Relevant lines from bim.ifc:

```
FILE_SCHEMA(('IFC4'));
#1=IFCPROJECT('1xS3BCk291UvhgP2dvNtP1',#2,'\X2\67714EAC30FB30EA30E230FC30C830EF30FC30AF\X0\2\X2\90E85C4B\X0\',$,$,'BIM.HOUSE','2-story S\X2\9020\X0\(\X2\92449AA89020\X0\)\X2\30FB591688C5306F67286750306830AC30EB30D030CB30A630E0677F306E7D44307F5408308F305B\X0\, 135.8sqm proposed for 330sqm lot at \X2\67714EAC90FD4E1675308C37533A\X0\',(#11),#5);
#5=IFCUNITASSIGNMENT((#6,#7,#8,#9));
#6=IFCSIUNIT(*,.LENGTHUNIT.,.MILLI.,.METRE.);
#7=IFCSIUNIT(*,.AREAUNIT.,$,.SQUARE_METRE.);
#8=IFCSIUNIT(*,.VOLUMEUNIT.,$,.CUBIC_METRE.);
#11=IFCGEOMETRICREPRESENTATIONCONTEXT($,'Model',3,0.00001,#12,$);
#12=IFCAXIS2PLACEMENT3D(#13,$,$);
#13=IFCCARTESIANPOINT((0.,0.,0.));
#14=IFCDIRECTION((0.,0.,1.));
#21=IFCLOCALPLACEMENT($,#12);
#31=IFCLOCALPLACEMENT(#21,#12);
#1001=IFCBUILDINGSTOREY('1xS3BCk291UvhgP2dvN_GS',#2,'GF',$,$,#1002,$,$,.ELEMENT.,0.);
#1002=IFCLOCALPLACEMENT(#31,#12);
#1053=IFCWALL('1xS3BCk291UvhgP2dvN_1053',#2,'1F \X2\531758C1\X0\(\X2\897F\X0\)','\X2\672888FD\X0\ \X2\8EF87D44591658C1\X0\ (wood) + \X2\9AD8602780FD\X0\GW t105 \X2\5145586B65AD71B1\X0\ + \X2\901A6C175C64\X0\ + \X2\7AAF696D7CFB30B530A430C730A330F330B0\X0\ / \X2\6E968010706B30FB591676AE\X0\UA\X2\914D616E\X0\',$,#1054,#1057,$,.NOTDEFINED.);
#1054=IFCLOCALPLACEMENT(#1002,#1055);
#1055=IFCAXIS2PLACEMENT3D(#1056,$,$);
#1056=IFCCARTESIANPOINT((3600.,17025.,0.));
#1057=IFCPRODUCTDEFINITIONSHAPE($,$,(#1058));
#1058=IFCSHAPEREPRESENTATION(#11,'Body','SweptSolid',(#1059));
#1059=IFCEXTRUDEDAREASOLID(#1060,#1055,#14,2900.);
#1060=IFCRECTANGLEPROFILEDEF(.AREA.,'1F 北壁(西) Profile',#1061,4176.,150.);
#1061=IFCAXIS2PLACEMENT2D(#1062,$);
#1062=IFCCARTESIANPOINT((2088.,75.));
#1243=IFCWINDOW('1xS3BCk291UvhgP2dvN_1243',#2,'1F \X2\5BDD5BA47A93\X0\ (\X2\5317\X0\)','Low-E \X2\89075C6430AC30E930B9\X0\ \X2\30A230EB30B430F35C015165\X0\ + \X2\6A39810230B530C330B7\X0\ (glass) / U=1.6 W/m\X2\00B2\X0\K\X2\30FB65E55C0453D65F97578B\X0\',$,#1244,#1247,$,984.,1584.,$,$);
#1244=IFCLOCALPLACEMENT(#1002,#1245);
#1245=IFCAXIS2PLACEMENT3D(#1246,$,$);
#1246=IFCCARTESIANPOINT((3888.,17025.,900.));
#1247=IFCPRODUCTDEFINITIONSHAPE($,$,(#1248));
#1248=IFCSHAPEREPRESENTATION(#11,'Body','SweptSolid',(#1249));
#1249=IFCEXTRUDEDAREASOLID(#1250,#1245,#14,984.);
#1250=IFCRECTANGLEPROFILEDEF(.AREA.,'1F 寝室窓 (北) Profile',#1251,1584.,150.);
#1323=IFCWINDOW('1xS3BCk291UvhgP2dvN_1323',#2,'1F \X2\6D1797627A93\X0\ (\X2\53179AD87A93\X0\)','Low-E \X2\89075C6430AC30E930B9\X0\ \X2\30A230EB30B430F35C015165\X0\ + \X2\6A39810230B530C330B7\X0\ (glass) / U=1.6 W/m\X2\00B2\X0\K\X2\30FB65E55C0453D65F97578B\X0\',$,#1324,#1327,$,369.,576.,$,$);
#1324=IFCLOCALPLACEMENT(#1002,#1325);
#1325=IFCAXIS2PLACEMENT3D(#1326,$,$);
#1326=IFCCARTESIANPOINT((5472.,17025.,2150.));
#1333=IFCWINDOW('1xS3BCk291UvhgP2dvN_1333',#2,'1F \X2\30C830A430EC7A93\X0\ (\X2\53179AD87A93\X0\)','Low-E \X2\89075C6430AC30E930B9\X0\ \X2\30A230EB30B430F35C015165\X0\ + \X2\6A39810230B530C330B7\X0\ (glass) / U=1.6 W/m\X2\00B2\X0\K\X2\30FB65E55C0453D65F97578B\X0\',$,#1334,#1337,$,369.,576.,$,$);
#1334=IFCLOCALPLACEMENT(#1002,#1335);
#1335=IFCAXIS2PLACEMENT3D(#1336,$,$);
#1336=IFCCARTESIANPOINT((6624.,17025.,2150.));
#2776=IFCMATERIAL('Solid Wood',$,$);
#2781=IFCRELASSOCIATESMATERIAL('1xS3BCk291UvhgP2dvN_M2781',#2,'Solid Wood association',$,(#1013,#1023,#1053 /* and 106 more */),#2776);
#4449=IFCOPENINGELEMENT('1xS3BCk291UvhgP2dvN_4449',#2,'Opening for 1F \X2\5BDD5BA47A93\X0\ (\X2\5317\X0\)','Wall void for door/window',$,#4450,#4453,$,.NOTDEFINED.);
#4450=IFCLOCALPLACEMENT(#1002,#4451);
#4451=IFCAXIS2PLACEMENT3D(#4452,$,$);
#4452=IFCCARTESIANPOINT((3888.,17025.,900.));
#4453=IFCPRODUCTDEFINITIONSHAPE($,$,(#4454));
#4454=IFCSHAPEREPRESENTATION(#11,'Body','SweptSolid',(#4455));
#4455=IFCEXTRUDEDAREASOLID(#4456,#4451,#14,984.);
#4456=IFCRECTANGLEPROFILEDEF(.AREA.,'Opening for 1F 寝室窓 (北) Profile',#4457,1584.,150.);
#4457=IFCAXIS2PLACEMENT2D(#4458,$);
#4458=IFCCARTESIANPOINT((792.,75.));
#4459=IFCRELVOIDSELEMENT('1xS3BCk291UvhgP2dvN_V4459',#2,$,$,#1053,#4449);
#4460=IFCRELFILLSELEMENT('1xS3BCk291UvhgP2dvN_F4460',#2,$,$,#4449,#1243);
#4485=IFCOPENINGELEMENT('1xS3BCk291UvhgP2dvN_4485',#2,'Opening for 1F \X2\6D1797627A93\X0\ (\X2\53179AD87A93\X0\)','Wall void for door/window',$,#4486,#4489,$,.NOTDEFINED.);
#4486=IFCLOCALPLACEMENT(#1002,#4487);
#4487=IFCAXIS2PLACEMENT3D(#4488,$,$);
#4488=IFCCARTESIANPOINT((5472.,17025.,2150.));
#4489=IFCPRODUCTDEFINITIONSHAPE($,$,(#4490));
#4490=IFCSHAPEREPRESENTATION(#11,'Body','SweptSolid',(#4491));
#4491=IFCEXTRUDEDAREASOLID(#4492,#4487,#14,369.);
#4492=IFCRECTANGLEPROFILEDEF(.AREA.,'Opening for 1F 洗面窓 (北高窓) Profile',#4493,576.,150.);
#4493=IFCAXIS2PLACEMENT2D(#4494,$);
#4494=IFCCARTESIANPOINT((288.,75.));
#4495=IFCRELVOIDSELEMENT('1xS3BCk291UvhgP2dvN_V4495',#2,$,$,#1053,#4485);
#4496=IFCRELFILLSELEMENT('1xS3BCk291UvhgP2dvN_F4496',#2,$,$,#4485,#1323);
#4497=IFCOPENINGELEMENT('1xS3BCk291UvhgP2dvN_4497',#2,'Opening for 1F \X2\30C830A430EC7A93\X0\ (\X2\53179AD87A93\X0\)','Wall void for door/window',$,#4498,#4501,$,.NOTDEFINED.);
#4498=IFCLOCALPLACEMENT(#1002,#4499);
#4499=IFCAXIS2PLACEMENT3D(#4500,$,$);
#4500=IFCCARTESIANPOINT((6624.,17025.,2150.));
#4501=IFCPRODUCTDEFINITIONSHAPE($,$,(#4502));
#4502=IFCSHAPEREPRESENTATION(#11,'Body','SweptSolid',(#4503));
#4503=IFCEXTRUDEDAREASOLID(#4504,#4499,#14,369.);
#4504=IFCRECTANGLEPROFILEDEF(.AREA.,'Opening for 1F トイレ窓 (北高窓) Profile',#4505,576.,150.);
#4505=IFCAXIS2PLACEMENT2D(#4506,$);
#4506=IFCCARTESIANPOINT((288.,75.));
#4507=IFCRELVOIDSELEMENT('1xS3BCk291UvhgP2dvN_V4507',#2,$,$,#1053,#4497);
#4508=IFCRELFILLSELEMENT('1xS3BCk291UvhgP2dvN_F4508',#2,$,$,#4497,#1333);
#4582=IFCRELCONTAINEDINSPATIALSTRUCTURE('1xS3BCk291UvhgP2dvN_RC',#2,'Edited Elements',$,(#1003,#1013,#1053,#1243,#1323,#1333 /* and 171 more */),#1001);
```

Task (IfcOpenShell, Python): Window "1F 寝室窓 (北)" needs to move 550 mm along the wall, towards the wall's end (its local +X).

```python
import ifcopenshell
import ifcopenshell.api.geometry
import ifcopenshell.util.placement

model = ifcopenshell.open("bim.ifc")

window = model.by_guid("1xS3BCk291UvhgP2dvN_1243")
opening = window.FillsVoids[0].RelatingOpeningElement
wall = opening.VoidsElements[0].RelatingBuildingElement

wall_matrix = ifcopenshell.util.placement.get_local_placement(wall.ObjectPlacement)
shift = wall_matrix[:3, 0] * 550.0
before = ifcopenshell.util.placement.get_local_placement(window.ObjectPlacement)[:3, 3].copy()

# The window is not placed relative to its opening, so move both.
for product in (opening, window):
    matrix = ifcopenshell.util.placement.get_local_placement(product.ObjectPlacement)
    matrix[:3, 3] += shift
    ifcopenshell.api.geometry.edit_object_placement(model, product=product, matrix=matrix, is_si=False)

after = ifcopenshell.util.placement.get_local_placement(window.ObjectPlacement)[:3, 3]
print("window moved by", (after - before).round(3) + 0.0)

model.write("bim_rev.ifc")
```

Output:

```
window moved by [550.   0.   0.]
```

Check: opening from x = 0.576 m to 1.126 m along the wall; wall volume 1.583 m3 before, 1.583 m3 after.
